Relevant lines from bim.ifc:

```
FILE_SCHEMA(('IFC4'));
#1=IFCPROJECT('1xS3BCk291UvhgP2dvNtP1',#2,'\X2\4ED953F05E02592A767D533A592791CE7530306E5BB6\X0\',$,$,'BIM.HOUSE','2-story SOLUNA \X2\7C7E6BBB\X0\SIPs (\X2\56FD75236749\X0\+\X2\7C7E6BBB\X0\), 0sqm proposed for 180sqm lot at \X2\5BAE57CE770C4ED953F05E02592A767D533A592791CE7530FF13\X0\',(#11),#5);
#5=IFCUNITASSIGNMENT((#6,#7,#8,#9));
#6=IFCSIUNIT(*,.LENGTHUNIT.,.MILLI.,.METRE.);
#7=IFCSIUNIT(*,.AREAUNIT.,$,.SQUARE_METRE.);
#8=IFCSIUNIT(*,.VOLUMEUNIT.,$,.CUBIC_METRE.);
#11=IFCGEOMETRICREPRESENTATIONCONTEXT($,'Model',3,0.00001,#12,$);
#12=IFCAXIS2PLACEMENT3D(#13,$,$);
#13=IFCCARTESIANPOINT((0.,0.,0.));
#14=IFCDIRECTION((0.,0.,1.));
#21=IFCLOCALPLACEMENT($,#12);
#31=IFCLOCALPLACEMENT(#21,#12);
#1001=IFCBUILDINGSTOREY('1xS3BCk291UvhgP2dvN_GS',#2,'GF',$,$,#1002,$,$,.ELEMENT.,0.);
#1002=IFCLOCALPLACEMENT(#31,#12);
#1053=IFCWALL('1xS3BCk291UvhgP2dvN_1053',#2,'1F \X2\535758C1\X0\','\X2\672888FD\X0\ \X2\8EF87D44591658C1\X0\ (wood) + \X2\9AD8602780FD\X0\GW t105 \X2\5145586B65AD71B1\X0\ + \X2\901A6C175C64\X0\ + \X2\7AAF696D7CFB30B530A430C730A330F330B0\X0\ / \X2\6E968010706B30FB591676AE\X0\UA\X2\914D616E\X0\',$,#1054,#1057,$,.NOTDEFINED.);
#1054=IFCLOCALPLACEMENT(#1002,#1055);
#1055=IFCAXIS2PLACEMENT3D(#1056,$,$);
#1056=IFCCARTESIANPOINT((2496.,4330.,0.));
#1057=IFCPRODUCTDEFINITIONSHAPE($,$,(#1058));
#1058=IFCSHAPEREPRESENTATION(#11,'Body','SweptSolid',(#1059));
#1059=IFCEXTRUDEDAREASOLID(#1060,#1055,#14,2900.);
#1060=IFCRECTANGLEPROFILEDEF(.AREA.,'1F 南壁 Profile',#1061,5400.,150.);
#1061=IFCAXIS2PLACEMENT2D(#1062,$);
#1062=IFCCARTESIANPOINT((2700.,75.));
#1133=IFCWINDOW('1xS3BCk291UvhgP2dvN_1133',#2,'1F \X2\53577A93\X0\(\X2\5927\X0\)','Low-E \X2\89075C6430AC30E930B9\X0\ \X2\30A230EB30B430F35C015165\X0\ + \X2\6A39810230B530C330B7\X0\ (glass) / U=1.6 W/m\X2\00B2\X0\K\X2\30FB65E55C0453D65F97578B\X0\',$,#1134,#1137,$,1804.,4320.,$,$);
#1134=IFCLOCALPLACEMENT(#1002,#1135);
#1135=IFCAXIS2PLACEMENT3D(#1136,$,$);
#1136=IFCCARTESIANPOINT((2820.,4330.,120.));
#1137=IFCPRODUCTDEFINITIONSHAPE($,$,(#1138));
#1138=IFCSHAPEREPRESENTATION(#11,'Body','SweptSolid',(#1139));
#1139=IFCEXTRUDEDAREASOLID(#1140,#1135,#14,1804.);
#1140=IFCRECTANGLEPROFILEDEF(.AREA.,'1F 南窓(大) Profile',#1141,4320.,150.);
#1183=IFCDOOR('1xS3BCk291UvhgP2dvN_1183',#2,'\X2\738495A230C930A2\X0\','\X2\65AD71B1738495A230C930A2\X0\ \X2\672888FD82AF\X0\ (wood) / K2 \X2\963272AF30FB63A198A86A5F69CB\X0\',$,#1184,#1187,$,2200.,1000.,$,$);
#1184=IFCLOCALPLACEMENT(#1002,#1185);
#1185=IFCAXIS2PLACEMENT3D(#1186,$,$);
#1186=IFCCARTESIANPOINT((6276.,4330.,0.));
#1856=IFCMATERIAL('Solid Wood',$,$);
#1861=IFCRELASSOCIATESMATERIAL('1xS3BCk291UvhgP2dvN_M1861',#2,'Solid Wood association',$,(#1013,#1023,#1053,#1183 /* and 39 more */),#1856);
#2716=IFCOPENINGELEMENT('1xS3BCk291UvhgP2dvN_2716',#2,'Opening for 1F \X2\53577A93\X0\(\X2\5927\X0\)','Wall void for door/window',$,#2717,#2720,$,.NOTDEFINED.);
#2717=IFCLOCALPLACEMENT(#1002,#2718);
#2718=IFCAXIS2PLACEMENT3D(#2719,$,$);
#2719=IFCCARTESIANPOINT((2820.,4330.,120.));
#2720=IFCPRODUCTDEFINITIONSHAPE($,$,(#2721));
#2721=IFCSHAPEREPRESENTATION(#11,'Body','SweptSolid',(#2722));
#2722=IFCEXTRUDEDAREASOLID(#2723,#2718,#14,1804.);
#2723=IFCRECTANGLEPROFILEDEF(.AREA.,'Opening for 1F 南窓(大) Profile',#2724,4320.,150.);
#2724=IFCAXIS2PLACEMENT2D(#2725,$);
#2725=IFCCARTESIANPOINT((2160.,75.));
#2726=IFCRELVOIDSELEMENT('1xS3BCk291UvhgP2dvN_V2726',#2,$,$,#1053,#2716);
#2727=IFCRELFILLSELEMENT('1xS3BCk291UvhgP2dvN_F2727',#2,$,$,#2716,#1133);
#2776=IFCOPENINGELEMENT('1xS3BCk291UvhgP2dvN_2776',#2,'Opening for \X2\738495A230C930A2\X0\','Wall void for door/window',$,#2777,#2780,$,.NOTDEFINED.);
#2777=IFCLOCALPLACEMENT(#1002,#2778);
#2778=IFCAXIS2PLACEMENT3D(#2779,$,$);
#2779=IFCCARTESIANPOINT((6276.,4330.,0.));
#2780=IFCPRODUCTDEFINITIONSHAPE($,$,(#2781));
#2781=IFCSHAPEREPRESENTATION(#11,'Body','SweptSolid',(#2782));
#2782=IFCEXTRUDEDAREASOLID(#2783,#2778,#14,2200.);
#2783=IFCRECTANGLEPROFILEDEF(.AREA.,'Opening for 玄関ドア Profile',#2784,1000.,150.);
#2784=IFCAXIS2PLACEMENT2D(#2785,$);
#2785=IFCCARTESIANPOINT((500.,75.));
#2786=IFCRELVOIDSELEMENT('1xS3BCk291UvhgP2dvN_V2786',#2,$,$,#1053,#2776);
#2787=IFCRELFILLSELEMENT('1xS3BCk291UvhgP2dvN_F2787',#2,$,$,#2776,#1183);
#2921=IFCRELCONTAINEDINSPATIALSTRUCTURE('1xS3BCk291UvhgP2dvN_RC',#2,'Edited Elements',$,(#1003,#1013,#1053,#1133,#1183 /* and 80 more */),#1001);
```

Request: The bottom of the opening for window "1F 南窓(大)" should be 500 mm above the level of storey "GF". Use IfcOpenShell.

```python
import numpy as np
import ifcopenshell
import ifcopenshell.api.geometry
import ifcopenshell.geom
import ifcopenshell.util.element
import ifcopenshell.util.placement
import ifcopenshell.util.shape
import ifcopenshell.util.unit

model = ifcopenshell.open("bim.ifc")
unit_scale = ifcopenshell.util.unit.calculate_unit_scale(model)

window = model.by_id(1133)
opening = window.FillsVoids[0].RelatingOpeningElement
storey = ifcopenshell.util.element.get_container(window, ifc_class="IfcBuildingStorey")
level = ifcopenshell.util.placement.get_local_placement(storey.ObjectPlacement)[2, 3]

# The opening's origin need not be at the sill, so measure its lowest point.
shape = ifcopenshell.geom.create_shape(ifcopenshell.geom.settings(), opening)
bottom = ifcopenshell.util.shape.get_shape_bottom_elevation(shape, shape.geometry) / unit_scale
dz = level + 0.5 / unit_scale - bottom

shift = np.array([0.0, 0.0, dz])
# The window is not placed relative to its opening, so move both.
for product in (opening, window):
    matrix = ifcopenshell.util.placement.get_local_placement(product.ObjectPlacement)
    matrix[:3, 3] += shift
    ifcopenshell.api.geometry.edit_object_placement(model, product=product, matrix=matrix, is_si=False)

print(f"moved by {dz * unit_scale:+.3f} m")

model.write("bim_updated.ifc")
```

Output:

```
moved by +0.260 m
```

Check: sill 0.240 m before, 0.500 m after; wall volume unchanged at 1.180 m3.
